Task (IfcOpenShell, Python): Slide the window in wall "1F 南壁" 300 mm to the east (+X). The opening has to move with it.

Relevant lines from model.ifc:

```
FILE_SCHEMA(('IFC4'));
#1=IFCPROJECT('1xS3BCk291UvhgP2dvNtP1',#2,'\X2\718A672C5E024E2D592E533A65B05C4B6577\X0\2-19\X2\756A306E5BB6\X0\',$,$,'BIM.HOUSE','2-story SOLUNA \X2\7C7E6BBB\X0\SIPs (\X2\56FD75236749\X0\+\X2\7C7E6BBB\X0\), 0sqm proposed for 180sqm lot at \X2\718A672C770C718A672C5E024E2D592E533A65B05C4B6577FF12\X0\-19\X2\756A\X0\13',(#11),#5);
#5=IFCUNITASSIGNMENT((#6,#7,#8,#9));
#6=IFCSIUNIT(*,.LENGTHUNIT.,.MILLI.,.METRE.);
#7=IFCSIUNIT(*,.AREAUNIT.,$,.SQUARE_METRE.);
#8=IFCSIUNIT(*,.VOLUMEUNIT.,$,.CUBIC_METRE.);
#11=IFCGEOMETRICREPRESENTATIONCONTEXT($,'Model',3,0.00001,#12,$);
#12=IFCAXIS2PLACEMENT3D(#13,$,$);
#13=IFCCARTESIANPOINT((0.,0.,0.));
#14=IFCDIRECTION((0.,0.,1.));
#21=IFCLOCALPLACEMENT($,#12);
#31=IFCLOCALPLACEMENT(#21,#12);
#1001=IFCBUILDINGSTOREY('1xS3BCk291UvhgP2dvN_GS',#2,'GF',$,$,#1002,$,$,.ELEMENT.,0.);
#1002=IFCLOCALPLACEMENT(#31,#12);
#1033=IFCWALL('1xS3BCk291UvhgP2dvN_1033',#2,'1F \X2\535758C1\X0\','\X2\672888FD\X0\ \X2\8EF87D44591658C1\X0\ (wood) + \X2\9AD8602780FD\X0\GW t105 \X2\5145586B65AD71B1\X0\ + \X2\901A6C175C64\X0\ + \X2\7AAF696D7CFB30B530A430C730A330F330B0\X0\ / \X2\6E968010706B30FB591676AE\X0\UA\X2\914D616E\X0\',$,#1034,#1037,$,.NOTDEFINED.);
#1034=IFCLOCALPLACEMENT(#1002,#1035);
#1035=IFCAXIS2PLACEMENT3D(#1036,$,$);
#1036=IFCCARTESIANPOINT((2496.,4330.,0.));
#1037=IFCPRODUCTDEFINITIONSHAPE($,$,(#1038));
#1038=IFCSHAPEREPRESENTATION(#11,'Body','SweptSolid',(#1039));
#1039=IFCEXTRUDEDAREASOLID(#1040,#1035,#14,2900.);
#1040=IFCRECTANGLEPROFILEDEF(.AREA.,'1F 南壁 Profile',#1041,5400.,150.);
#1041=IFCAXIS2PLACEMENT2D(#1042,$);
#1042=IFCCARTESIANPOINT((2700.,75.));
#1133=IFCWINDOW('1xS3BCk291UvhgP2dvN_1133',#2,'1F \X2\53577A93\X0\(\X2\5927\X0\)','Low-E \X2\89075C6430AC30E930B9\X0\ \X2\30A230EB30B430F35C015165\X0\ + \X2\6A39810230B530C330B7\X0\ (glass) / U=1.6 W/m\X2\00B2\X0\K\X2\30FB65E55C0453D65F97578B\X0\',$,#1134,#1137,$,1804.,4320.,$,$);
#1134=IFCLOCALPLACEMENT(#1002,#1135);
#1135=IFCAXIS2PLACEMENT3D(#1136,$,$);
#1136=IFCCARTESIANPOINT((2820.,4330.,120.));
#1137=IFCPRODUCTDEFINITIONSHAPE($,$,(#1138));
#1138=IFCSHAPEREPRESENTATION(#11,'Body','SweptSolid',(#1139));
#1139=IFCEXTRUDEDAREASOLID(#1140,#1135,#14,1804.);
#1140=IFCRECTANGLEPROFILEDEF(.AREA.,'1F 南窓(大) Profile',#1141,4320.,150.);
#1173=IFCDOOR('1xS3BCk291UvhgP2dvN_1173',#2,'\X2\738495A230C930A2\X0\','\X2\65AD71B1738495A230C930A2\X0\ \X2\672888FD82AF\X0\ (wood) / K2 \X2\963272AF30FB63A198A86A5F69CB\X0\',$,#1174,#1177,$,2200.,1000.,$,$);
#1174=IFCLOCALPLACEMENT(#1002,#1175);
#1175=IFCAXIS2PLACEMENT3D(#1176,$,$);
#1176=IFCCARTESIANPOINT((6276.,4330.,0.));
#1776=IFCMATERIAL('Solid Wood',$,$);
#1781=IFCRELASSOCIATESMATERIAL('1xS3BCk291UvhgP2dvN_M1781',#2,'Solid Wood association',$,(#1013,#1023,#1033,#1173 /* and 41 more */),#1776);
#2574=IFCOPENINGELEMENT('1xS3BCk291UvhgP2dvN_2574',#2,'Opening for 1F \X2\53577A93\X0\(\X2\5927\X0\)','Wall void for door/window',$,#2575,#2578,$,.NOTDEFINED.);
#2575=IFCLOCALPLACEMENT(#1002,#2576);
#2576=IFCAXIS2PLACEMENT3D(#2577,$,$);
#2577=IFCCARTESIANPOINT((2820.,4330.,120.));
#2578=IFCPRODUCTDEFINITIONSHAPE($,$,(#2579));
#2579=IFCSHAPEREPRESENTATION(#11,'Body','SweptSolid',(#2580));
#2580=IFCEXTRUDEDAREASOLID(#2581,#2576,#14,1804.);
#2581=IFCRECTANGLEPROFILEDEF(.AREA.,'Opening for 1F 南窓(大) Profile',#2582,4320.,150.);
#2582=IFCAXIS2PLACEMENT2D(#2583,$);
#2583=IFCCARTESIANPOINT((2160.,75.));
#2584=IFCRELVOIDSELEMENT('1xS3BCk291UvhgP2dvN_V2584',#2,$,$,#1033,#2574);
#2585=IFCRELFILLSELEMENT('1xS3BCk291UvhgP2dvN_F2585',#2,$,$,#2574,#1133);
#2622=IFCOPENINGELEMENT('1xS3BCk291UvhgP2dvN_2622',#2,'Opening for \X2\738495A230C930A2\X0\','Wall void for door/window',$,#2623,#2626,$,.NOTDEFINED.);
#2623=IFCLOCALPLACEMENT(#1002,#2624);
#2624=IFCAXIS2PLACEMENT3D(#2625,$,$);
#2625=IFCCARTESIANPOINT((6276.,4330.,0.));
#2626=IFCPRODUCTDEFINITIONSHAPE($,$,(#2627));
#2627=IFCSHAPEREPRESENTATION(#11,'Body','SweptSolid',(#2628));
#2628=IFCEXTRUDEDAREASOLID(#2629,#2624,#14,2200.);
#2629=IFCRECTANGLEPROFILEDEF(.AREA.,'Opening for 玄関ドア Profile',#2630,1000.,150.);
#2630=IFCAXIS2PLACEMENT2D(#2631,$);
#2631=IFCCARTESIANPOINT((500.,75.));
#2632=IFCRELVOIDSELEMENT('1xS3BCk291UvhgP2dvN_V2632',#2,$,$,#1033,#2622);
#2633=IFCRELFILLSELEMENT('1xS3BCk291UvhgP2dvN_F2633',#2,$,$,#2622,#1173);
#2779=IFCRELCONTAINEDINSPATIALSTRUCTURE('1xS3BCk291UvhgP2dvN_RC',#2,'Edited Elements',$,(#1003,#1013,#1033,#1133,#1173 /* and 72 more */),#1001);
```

```python
import ifcopenshell
import ifcopenshell.api.geometry
import ifcopenshell.util.placement
import ifcopenshell.util.unit

model = ifcopenshell.open("model.ifc")
unit_scale = ifcopenshell.util.unit.calculate_unit_scale(model)

window = model.by_id(1133)
opening = window.FillsVoids[0].RelatingOpeningElement
wall = opening.VoidsElements[0].RelatingBuildingElement

wall_matrix = ifcopenshell.util.placement.get_local_placement(wall.ObjectPlacement)
shift = wall_matrix[:3, 0] * 0.3 / unit_scale
before = ifcopenshell.util.placement.get_local_placement(window.ObjectPlacement)[:3, 3].copy()

# The window is not placed relative to its opening, so move both.
for product in (opening, window):
    matrix = ifcopenshell.util.placement.get_local_placement(product.ObjectPlacement)
    matrix[:3, 3] += shift
    ifcopenshell.api.geometry.edit_object_placement(model, product=product, matrix=matrix, is_si=False)

after = ifcopenshell.util.placement.get_local_placement(window.ObjectPlacement)[:3, 3]
print("window moved by", (after - before).round(3) + 0.0)

model.write("model_updated.ifc")
```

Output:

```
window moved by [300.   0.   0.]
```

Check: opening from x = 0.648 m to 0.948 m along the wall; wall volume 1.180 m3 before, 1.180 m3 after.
